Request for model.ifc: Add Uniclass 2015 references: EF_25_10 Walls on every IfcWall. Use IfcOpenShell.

First a look at what the model holds.

```python
import ifcopenshell

model = ifcopenshell.open("model.ifc")
print(model.schema)
print("classifications:", [c.Name for c in model.by_type("IfcClassification")])
for ifc_class in ("IfcDoor", "IfcRoof", "IfcStair", "IfcWall", "IfcWindow"):
    print(ifc_class, len(model.by_type(ifc_class)))
```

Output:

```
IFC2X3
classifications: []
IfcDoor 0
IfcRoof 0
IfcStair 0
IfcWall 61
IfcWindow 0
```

```python
import ifcopenshell
import ifcopenshell.api.classification

model = ifcopenshell.open("model.ifc")

# IFC2X3 requires Source and Edition and has no link from the project to the system.
system = model.create_entity("IfcClassification", Source="NBS", Edition="2015", Name="Uniclass 2015")

codes = {
    "IfcWall": ("EF_25_10", "Walls"),
}
for ifc_class, (code, name) in codes.items():
    products = model.by_type(ifc_class)
    ifcopenshell.api.classification.add_reference(
        model, products=products, classification=system, identification=code, name=name
    )
    print(code, len(products))

model.write("model-out.ifc")
```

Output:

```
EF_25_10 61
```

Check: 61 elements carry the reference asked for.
